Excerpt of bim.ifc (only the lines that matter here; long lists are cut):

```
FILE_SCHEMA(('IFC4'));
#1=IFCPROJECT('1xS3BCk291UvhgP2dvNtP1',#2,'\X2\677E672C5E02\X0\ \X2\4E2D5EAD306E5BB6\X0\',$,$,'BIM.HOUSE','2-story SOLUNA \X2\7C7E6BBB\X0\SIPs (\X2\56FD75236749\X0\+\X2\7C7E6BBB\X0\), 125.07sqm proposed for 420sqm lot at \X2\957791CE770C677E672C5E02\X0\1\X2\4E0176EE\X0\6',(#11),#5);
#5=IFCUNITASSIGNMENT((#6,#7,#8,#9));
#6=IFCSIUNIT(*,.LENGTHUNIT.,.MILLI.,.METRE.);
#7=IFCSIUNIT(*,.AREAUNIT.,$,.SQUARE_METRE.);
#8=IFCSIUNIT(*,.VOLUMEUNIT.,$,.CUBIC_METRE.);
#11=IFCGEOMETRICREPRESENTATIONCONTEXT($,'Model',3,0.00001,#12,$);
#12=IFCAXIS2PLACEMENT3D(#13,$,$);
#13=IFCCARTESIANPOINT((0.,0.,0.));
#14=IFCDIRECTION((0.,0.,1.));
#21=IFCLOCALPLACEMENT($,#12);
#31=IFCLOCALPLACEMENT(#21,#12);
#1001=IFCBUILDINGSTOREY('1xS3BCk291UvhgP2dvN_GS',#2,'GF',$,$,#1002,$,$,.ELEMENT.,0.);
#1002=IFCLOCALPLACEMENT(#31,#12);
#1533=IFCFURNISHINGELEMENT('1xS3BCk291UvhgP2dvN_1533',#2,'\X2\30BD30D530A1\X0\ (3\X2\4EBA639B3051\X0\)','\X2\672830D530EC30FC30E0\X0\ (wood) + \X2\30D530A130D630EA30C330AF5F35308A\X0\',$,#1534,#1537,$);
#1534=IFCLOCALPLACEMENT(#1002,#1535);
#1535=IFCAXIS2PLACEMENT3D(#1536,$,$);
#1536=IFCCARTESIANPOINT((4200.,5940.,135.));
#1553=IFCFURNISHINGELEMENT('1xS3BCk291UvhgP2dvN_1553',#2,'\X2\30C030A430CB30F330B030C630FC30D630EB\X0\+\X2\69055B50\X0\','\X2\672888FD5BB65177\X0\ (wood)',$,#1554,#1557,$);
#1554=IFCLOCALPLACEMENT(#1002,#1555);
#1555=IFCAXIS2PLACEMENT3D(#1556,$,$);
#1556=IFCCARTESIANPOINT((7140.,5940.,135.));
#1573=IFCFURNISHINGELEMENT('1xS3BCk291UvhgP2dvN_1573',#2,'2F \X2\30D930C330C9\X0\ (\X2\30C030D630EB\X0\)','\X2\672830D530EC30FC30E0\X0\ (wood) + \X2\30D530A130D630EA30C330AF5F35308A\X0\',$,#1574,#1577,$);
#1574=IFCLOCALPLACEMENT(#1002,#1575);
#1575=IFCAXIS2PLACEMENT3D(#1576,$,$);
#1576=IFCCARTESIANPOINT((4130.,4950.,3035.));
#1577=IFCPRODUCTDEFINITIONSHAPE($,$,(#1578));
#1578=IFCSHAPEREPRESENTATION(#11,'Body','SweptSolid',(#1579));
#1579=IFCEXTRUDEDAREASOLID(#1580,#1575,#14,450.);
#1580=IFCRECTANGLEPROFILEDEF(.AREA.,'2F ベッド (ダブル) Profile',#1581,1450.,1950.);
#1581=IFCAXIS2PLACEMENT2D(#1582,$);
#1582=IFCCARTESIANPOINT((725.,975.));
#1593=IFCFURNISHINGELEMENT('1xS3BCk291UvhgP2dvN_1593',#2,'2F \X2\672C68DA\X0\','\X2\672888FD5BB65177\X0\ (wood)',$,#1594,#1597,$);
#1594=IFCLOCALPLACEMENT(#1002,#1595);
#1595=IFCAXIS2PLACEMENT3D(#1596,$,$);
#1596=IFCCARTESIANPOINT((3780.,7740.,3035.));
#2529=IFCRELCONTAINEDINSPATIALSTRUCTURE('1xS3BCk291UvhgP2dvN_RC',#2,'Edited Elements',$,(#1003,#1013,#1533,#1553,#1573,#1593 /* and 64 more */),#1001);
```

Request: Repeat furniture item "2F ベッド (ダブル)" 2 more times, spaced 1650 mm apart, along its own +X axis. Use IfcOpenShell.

```python
import ifcopenshell
import ifcopenshell.api.geometry
import ifcopenshell.api.root
import ifcopenshell.util.element
import ifcopenshell.util.placement
import ifcopenshell.util.unit

model = ifcopenshell.open("bim.ifc")
unit_scale = ifcopenshell.util.unit.calculate_unit_scale(model)


def reuse_history(source, copy):
    """copy_class also copies each property set's owner history, people and application; keep the originals."""
    for rel in copy.IsDefinedBy:
        if rel.is_a("IfcRelDefinesByProperties") and (history := rel.RelatingPropertyDefinition.OwnerHistory):
            rel.RelatingPropertyDefinition.OwnerHistory = source.OwnerHistory
            ifcopenshell.util.element.remove_deep2(model, history)


source = model.by_guid("1xS3BCk291UvhgP2dvN_1573")
base = ifcopenshell.util.placement.get_local_placement(source.ObjectPlacement)
step = base[:3, 0] * 1.65 / unit_scale

for i in range(1, 3):
    copy = ifcopenshell.api.root.copy_class(model, product=source)
    copy.Representation = ifcopenshell.util.element.copy_deep(
        model, source.Representation, exclude=["IfcGeometricRepresentationContext", "IfcRepresentationMap"]
    )
    reuse_history(source, copy)
    matrix = base.copy()
    matrix[:3, 3] += i * step
    print("added at", matrix[:3, 3].round(3) + 0.0)
    ifcopenshell.api.geometry.edit_object_placement(model, product=copy, matrix=matrix, is_si=False)

model.write("bim_v2.ifc")
```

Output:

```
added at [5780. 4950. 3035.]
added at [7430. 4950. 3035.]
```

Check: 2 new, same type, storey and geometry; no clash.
